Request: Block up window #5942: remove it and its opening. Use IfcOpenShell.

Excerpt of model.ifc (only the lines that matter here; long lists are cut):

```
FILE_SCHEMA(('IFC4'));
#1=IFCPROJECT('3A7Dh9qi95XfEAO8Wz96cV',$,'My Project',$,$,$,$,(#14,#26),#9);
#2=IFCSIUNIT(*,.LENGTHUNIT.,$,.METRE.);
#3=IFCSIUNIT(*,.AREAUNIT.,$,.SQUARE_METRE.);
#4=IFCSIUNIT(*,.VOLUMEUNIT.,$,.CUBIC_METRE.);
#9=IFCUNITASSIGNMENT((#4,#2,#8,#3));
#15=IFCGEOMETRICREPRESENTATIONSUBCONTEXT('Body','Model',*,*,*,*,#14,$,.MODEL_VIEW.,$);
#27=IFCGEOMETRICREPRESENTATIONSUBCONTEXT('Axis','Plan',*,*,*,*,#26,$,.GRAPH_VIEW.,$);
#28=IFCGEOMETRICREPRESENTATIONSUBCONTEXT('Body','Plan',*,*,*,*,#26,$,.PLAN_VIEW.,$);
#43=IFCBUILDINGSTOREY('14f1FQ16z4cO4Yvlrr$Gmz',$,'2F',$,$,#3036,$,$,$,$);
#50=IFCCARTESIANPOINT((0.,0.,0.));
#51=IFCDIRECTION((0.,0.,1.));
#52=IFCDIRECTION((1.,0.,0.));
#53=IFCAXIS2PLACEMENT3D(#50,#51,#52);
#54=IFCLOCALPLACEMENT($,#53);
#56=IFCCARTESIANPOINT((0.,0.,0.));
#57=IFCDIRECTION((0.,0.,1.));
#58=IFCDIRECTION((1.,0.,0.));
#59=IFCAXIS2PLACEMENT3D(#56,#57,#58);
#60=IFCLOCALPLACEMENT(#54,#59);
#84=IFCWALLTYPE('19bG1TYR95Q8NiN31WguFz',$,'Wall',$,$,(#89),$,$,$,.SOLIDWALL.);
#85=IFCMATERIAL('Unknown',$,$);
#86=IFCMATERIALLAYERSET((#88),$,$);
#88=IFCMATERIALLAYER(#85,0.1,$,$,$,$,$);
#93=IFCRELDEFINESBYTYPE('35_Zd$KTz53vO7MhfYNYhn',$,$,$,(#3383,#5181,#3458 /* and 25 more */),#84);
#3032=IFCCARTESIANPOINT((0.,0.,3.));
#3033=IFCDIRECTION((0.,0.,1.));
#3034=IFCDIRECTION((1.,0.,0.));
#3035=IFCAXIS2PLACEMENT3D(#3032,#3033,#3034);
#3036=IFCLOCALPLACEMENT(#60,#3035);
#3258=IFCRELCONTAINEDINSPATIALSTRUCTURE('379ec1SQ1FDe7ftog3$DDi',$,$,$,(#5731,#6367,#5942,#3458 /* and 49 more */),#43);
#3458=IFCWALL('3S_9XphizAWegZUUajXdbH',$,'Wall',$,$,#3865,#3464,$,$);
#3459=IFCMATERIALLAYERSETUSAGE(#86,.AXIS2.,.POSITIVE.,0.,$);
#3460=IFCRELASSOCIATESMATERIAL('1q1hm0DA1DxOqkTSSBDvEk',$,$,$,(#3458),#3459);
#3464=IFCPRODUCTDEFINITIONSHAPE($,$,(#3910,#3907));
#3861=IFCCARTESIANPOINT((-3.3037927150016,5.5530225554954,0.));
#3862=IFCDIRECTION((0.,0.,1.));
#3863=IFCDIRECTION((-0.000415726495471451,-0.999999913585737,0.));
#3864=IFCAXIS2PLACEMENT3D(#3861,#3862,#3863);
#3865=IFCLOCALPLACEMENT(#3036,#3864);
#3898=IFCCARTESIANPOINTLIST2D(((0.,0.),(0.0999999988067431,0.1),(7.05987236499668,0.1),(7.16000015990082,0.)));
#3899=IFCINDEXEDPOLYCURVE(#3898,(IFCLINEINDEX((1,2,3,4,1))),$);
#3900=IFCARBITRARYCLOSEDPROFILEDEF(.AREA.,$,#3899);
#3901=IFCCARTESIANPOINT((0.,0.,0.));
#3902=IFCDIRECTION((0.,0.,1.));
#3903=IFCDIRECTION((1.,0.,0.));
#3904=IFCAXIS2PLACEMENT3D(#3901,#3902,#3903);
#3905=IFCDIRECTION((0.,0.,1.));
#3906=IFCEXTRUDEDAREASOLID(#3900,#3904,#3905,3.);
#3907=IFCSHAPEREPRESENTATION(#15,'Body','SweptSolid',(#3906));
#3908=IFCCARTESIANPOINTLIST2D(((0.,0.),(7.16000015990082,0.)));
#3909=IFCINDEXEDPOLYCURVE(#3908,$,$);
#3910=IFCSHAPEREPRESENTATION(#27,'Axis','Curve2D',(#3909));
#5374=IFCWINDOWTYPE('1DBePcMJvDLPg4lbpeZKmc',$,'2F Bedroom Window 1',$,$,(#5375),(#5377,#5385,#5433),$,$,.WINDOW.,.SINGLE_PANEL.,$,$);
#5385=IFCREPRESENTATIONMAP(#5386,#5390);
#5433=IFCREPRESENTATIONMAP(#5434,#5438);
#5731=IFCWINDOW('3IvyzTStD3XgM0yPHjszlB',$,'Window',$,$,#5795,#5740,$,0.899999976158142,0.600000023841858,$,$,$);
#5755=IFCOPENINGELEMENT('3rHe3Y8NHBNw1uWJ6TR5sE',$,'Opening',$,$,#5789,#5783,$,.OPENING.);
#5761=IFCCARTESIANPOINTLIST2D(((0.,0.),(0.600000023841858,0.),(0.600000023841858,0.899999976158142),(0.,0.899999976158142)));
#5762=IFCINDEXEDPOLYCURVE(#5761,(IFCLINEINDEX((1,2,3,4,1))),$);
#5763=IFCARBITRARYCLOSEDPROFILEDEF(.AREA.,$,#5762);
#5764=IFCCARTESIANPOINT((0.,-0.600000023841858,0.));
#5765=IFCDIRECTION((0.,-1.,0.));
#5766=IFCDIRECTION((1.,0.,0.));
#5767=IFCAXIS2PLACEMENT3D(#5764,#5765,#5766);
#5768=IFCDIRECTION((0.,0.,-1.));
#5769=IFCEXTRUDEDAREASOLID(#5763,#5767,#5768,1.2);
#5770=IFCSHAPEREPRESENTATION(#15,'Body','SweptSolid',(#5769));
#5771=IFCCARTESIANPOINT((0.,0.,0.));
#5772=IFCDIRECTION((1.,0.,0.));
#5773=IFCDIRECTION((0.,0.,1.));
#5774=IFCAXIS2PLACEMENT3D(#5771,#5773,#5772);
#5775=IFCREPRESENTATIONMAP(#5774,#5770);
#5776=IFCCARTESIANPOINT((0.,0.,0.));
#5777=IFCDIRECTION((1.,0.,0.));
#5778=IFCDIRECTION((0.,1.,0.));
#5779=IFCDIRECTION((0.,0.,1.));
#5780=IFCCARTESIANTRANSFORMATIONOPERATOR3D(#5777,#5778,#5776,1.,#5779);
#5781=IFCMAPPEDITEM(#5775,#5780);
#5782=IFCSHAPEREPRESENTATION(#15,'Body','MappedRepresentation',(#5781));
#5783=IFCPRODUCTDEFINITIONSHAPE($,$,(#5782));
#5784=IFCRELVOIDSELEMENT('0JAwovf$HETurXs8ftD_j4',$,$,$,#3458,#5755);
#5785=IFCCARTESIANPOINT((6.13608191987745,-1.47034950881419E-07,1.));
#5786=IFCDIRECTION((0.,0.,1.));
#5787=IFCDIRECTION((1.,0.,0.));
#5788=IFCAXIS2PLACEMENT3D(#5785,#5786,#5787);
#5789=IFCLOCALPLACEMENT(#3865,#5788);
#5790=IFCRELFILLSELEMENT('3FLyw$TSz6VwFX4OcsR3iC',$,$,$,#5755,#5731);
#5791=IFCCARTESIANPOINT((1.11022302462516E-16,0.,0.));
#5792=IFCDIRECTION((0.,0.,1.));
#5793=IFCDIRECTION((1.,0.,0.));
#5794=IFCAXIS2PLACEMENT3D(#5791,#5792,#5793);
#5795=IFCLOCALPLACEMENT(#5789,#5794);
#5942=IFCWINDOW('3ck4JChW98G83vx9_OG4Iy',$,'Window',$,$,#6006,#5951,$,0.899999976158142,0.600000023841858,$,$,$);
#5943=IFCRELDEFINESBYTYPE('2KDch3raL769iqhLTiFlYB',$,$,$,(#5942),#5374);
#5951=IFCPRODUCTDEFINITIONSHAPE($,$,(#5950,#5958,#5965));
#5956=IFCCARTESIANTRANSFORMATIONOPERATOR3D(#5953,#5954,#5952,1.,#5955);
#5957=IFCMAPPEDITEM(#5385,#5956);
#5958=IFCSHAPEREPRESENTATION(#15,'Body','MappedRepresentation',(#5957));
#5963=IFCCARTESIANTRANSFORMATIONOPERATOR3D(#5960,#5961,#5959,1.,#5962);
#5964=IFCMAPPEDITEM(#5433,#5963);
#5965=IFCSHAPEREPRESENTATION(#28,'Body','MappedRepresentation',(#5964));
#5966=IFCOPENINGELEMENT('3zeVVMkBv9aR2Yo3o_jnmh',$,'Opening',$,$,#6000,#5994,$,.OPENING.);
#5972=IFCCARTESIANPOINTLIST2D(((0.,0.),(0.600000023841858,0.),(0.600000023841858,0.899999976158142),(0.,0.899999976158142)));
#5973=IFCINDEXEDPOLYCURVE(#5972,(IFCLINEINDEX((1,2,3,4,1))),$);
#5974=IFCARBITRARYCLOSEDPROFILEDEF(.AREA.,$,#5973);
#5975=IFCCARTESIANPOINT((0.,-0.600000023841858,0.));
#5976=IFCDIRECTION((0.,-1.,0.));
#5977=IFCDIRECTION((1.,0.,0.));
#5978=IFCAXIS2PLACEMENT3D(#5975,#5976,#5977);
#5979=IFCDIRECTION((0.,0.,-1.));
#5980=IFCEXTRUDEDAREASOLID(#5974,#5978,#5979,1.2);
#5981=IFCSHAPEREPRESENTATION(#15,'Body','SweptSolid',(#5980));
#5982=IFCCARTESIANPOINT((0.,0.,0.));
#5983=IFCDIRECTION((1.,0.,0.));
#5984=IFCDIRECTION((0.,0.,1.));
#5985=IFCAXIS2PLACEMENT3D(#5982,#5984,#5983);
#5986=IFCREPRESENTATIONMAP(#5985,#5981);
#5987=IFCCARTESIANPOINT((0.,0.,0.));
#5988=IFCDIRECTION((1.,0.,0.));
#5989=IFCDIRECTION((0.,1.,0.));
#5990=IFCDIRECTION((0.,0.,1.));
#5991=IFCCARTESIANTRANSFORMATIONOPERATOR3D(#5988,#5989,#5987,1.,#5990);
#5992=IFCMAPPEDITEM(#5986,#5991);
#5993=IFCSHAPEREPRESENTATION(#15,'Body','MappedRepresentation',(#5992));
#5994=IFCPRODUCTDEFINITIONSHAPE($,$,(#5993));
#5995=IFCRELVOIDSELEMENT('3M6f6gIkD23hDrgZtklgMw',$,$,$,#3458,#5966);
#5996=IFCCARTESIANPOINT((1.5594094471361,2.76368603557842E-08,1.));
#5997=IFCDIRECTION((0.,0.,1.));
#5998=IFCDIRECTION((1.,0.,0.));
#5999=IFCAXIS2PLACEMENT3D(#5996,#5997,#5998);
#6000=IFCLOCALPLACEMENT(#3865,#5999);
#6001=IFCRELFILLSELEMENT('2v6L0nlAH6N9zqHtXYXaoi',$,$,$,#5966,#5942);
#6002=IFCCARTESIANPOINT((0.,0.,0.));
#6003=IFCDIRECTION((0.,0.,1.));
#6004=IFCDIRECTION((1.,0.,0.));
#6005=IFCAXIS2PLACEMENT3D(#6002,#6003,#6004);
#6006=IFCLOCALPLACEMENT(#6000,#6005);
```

```python
import ifcopenshell
import ifcopenshell.api.feature
import ifcopenshell.api.root
import ifcopenshell.geom
import ifcopenshell.util.shape

model = ifcopenshell.open("model.ifc")
settings = ifcopenshell.geom.settings()


def volume(element):
    """Net volume in cubic metres, openings subtracted."""
    shape = ifcopenshell.geom.create_shape(settings, element)
    return ifcopenshell.util.shape.get_volume(shape.geometry)


window = model.by_guid("3ck4JChW98G83vx9_OG4Iy")
opening = window.FillsVoids[0].RelatingOpeningElement
wall = opening.VoidsElements[0].RelatingBuildingElement
before = volume(wall)

ifcopenshell.api.root.remove_product(model, product=window)
ifcopenshell.api.feature.remove_feature(model, feature=opening)

after = volume(wall)

print(f"wall volume {before:.3f} -> {after:.3f} m3")

model.write("model_updated.ifc")
```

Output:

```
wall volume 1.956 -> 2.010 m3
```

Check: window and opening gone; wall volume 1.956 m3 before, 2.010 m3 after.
